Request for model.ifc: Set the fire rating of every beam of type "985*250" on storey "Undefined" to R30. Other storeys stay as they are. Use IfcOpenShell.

First a look at what the model holds.

```python
import ifcopenshell
import ifcopenshell.util.element

model = ifcopenshell.open("model.ifc")
print(model.schema)
storey = next(s for s in model.by_type("IfcBuildingStorey") if s.Name == "Undefined")
beams = [e for e in ifcopenshell.util.element.get_decomposition(storey) if e.is_a("IfcBeam")]
seen = {}
for e in beams:
    element_type = ifcopenshell.util.element.get_type(e)
    key = (element_type.Name if element_type != e and element_type else None, ifcopenshell.util.element.get_pset(e, "Pset_BeamCommon", "FireRating"))
    seen[key] = seen.get(key, 0) + 1
for (name, value), count in sorted(seen.items(), key=str):
    print(count, "x", name, "|", value)
```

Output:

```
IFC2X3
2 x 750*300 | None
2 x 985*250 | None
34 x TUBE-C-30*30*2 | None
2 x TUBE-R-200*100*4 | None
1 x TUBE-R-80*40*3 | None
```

```python
import ifcopenshell
import ifcopenshell.api.pset
import ifcopenshell.util.element

model = ifcopenshell.open("model.ifc")

storey = next(s for s in model.by_type("IfcBuildingStorey") if s.Name == "Undefined")
beams = [e for e in ifcopenshell.util.element.get_decomposition(storey) if e.is_a("IfcBeam")]

count = 0
for e in beams:
    element_type = ifcopenshell.util.element.get_type(e)
    if element_type in (None, e) or element_type.Name != "985*250":
        continue
    # add_pset returns the element's existing set when there is one.
    pset = ifcopenshell.api.pset.add_pset(model, product=e, name="Pset_BeamCommon")
    ifcopenshell.api.pset.edit_pset(model, pset=pset, properties={"FireRating": "R30"})
    count += 1

print(count, "beams updated")

model.write("model_rev.ifc")
```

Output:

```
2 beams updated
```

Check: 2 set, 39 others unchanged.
